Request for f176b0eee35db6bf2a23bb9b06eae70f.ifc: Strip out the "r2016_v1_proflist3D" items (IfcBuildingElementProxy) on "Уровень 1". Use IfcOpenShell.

First a look at what the model holds.

```python
import ifcopenshell
import ifcopenshell.util.element

model = ifcopenshell.open("f176b0eee35db6bf2a23bb9b06eae70f.ifc")
print(model.schema)
storey = next(s for s in model.by_type("IfcBuildingStorey") if s.Name == "Уровень 1")
proxies = [e for e in ifcopenshell.util.element.get_decomposition(storey) if e.is_a("IfcBuildingElementProxy")]
seen = {}
for e in proxies:
    element_type = ifcopenshell.util.element.get_type(e)
    name = element_type.Name if element_type not in (None, e) else None
    seen[name] = seen.get(name, 0) + 1
for name, count in sorted(seen.items(), key=str):
    print(count, "x", name)
```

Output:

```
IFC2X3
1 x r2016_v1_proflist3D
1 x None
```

```python
import ifcopenshell
import ifcopenshell.api.root
import ifcopenshell.util.element

model = ifcopenshell.open("f176b0eee35db6bf2a23bb9b06eae70f.ifc")

storey = next(s for s in model.by_type("IfcBuildingStorey") if s.Name == "Уровень 1")
proxies = [e for e in ifcopenshell.util.element.get_decomposition(storey) if e.is_a("IfcBuildingElementProxy")]
targets = [e for e in proxies if (t := ifcopenshell.util.element.get_type(e)) not in (None, e) and t.Name == "r2016_v1_proflist3D"]

for e in targets:
    ifcopenshell.api.root.remove_product(model, product=e)
print(len(targets), "removed")

model.write("f176b0eee35db6bf2a23bb9b06eae70f_updated.ifc")
```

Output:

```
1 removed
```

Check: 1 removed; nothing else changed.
